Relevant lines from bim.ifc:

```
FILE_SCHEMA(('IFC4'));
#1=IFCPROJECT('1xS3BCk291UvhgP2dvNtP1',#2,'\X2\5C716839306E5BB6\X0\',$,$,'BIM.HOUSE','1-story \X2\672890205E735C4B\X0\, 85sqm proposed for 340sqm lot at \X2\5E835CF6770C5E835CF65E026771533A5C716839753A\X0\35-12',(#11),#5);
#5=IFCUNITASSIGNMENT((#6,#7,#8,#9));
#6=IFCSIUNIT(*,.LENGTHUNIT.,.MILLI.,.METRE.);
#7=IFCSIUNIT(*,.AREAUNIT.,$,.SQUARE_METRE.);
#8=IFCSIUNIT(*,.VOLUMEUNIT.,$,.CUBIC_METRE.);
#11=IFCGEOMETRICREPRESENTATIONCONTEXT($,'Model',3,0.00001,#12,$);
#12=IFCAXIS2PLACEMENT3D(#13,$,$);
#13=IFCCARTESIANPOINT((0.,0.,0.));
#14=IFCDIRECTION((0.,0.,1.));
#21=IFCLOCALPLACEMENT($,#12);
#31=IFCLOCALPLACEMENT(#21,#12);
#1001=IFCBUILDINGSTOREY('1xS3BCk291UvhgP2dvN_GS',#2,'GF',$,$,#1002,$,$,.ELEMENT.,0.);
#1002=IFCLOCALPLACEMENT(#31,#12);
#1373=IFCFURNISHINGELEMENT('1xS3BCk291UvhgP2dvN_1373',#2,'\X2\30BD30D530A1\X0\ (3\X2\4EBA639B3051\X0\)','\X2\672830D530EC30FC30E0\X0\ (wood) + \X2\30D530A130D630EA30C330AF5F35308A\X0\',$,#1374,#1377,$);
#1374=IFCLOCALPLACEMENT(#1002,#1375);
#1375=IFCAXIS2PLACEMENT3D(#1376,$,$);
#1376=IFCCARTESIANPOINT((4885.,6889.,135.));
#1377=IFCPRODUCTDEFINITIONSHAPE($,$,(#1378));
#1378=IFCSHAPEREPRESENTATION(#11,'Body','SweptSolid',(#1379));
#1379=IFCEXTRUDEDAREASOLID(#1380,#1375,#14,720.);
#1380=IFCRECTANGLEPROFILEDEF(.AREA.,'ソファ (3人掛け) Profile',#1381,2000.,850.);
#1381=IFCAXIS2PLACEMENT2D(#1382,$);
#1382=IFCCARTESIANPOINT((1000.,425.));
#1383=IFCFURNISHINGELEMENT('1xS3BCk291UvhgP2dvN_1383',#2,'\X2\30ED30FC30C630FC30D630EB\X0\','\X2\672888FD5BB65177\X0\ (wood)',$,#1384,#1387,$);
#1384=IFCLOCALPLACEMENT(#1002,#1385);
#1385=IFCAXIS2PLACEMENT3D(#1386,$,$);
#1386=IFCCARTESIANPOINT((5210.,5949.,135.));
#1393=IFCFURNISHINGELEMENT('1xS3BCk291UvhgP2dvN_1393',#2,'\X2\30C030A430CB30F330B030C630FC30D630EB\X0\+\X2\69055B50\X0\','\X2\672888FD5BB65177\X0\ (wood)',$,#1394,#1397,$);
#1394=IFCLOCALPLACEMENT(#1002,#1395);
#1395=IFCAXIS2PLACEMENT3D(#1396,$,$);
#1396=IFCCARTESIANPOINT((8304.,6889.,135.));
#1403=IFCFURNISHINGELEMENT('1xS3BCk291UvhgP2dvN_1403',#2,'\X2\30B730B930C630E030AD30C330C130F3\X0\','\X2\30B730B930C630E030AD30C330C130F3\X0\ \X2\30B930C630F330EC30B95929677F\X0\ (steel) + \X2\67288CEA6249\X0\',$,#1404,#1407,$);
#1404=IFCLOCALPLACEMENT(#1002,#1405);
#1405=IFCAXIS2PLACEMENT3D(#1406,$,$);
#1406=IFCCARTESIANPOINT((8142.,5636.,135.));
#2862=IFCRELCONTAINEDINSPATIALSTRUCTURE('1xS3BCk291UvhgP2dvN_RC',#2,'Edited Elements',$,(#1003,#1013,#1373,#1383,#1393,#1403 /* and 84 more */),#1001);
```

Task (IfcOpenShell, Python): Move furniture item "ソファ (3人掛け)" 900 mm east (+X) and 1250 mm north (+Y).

```python
import ifcopenshell
import ifcopenshell.api.geometry
import ifcopenshell.util.placement
import ifcopenshell.util.unit

model = ifcopenshell.open("bim.ifc")
unit_scale = ifcopenshell.util.unit.calculate_unit_scale(model)

item = model.by_guid("1xS3BCk291UvhgP2dvN_1373")
matrix = ifcopenshell.util.placement.get_local_placement(item.ObjectPlacement)
matrix[0, 3] += 0.9 / unit_scale
matrix[1, 3] += 1.25 / unit_scale
ifcopenshell.api.geometry.edit_object_placement(model, product=item, matrix=matrix, is_si=False)

print(ifcopenshell.util.placement.get_local_placement(item.ObjectPlacement).round(3) + 0.0)

model.write("bim_rev.ifc")
```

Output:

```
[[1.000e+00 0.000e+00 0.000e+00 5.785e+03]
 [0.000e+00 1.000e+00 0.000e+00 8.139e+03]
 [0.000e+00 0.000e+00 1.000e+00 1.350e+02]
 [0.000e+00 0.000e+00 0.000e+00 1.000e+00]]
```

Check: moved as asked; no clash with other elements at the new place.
